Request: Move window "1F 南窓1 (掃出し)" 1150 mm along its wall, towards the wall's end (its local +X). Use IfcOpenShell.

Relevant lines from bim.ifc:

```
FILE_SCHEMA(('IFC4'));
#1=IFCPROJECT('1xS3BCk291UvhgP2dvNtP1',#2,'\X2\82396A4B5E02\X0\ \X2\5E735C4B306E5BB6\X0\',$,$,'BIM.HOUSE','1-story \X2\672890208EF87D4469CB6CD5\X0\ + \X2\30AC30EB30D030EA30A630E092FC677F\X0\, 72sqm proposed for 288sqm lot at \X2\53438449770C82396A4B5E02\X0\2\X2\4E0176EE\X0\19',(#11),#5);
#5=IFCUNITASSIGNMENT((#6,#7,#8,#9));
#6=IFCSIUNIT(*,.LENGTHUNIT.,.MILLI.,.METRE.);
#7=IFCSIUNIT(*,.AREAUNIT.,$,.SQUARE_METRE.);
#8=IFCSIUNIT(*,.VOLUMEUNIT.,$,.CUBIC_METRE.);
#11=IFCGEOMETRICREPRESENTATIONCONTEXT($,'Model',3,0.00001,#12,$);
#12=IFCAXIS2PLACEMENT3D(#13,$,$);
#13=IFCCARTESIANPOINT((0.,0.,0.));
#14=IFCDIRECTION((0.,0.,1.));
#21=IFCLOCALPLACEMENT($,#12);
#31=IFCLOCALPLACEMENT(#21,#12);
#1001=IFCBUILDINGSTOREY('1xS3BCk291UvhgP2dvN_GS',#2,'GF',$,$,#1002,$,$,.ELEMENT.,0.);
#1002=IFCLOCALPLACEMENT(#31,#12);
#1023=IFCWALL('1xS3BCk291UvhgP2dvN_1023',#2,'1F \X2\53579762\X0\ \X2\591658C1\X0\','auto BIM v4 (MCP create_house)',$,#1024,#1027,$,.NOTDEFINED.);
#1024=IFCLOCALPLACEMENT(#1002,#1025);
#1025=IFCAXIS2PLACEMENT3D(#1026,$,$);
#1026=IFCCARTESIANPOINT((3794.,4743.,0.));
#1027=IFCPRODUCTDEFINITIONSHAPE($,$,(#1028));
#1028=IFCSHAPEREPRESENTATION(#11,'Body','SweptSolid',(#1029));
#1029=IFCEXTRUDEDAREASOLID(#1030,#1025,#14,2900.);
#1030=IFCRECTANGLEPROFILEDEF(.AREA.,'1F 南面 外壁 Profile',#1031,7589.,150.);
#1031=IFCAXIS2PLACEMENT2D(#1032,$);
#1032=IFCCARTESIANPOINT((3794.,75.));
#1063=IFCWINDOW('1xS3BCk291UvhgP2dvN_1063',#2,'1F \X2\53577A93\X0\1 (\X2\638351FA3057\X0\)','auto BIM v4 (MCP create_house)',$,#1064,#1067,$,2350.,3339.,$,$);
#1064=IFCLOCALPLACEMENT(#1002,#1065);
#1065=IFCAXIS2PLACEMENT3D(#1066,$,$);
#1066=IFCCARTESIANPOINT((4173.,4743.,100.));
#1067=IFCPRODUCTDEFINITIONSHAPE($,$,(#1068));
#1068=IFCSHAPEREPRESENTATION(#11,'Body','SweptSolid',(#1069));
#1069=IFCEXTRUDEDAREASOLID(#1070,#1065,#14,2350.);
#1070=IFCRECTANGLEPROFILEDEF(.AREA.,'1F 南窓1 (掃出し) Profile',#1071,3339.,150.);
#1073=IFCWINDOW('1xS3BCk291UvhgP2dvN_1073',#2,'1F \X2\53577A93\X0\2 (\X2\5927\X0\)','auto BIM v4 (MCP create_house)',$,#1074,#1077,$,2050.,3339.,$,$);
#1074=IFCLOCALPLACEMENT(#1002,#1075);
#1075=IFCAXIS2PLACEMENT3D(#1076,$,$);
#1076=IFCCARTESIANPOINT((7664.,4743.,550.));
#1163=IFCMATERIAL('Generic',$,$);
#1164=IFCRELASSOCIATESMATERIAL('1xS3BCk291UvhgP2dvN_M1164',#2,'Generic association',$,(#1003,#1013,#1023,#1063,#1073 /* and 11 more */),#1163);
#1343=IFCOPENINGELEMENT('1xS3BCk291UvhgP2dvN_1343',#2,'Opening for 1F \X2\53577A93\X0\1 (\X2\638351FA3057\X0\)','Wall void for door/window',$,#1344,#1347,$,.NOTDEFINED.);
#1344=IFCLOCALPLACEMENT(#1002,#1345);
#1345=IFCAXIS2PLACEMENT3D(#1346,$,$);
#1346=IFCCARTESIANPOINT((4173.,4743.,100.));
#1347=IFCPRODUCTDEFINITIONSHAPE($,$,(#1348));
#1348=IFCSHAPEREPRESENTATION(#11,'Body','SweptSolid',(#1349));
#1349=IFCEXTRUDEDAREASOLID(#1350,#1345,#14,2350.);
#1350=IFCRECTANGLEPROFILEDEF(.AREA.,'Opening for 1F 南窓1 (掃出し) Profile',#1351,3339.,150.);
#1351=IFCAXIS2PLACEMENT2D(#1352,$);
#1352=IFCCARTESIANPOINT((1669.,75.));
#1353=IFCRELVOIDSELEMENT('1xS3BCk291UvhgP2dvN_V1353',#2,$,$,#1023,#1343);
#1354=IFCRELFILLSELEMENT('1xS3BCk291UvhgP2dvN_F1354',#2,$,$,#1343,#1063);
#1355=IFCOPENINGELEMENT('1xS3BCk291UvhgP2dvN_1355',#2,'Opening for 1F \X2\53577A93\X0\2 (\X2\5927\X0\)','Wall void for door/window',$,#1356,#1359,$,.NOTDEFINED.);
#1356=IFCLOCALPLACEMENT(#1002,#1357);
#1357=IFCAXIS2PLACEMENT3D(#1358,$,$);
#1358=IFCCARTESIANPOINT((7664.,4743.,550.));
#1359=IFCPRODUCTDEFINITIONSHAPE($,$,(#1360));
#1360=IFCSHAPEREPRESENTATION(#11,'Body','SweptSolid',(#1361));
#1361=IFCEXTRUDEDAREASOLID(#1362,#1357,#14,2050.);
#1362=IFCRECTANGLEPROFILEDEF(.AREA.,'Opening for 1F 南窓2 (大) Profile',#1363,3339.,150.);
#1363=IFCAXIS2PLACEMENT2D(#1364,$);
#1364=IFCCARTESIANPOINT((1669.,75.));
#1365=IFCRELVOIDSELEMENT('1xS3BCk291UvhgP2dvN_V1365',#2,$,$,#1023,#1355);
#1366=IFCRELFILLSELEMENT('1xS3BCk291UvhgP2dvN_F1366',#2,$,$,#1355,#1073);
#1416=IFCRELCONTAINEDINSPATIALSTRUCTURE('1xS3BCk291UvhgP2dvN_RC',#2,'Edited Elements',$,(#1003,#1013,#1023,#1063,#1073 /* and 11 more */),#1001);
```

```python
import ifcopenshell
import ifcopenshell.api.geometry
import ifcopenshell.util.placement
import ifcopenshell.util.unit

model = ifcopenshell.open("bim.ifc")
unit_scale = ifcopenshell.util.unit.calculate_unit_scale(model)

window = model.by_guid("1xS3BCk291UvhgP2dvN_1063")
opening = window.FillsVoids[0].RelatingOpeningElement
wall = opening.VoidsElements[0].RelatingBuildingElement

wall_matrix = ifcopenshell.util.placement.get_local_placement(wall.ObjectPlacement)
shift = wall_matrix[:3, 0] * 1.15 / unit_scale
before = ifcopenshell.util.placement.get_local_placement(window.ObjectPlacement)[:3, 3].copy()

# The window is not placed relative to its opening, so move both.
for product in (opening, window):
    matrix = ifcopenshell.util.placement.get_local_placement(product.ObjectPlacement)
    matrix[:3, 3] += shift
    ifcopenshell.api.geometry.edit_object_placement(model, product=product, matrix=matrix, is_si=False)

after = ifcopenshell.util.placement.get_local_placement(window.ObjectPlacement)[:3, 3]
print("window moved by", (after - before).round(3) + 0.0)

model.write("bim-out.ifc")
```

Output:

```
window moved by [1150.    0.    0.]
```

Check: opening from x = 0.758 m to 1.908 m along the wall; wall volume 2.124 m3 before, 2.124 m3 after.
